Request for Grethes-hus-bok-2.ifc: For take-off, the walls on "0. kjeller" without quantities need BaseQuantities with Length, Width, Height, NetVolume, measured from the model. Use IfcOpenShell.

First a look at what the model holds.

```python
import ifcopenshell
import ifcopenshell.util.element
import ifcopenshell.util.unit

model = ifcopenshell.open("Grethes-hus-bok-2.ifc")
print(model.schema)
for unit_type in ("LENGTHUNIT", "AREAUNIT", "VOLUMEUNIT"):
    print(unit_type, ifcopenshell.util.unit.calculate_unit_scale(model, unit_type))
storey = next(s for s in model.by_type("IfcBuildingStorey") if s.Name == "0. kjeller")
walls = [e for e in ifcopenshell.util.element.get_decomposition(storey) if e.is_a("IfcWall")]
for e in sorted(walls, key=lambda e: e.id()):
    print(e.id(), e.is_a(), e.Name, list(ifcopenshell.util.element.get_psets(e, qtos_only=True)), sep=" | ")
```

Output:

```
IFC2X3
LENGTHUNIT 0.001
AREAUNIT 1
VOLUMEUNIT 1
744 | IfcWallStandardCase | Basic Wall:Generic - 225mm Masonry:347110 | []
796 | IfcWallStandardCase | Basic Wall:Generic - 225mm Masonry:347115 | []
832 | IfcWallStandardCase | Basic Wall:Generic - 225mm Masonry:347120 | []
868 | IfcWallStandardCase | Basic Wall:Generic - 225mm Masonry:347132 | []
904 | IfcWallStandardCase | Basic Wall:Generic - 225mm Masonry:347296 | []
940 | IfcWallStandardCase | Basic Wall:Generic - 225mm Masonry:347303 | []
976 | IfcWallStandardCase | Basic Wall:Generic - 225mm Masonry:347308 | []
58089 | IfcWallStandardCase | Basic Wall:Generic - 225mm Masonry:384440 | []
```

```python
import ifcopenshell
import ifcopenshell.api.pset
import ifcopenshell.geom
import ifcopenshell.util.element
import ifcopenshell.util.shape
import ifcopenshell.util.unit

model = ifcopenshell.open("Grethes-hus-bok-2.ifc")
unit_scale = ifcopenshell.util.unit.calculate_unit_scale(model)
volume_scale = ifcopenshell.util.unit.calculate_unit_scale(model, "VOLUMEUNIT")
settings = ifcopenshell.geom.settings()

storey = next(s for s in model.by_type("IfcBuildingStorey") if s.Name == "0. kjeller")
walls = [e for e in ifcopenshell.util.element.get_decomposition(storey) if e.is_a("IfcWall")]

for e in sorted(walls, key=lambda e: e.id()):
    if ifcopenshell.util.element.get_psets(e, qtos_only=True, should_inherit=False):
        continue
    # Geometry comes back in metres, in the element's own axes.
    shape = ifcopenshell.geom.create_shape(settings, e)
    values = {
        "Length": ifcopenshell.util.shape.get_x(shape.geometry) / unit_scale,
        "Width": ifcopenshell.util.shape.get_y(shape.geometry) / unit_scale,
        "Height": ifcopenshell.util.shape.get_z(shape.geometry) / unit_scale,
        "NetVolume": ifcopenshell.util.shape.get_volume(shape.geometry) / volume_scale,
    }
    qto = ifcopenshell.api.pset.add_qto(model, product=e, name="BaseQuantities")
    ifcopenshell.api.pset.edit_qto(model, qto=qto, properties=values)
    print(e.id(), {k: round(v, 3) for k, v in values.items()})

model.write("Grethes-hus-bok-2-out.ifc")
```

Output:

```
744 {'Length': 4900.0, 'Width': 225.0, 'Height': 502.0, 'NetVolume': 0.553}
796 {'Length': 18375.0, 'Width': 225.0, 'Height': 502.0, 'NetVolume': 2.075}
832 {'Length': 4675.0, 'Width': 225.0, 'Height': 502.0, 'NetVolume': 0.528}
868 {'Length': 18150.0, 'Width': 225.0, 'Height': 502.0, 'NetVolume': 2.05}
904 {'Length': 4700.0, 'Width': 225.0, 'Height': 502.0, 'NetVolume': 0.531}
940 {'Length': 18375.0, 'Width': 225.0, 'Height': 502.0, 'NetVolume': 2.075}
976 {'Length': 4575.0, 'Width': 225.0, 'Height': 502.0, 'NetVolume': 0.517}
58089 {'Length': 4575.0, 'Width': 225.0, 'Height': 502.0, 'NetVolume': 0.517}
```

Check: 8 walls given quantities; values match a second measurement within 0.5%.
